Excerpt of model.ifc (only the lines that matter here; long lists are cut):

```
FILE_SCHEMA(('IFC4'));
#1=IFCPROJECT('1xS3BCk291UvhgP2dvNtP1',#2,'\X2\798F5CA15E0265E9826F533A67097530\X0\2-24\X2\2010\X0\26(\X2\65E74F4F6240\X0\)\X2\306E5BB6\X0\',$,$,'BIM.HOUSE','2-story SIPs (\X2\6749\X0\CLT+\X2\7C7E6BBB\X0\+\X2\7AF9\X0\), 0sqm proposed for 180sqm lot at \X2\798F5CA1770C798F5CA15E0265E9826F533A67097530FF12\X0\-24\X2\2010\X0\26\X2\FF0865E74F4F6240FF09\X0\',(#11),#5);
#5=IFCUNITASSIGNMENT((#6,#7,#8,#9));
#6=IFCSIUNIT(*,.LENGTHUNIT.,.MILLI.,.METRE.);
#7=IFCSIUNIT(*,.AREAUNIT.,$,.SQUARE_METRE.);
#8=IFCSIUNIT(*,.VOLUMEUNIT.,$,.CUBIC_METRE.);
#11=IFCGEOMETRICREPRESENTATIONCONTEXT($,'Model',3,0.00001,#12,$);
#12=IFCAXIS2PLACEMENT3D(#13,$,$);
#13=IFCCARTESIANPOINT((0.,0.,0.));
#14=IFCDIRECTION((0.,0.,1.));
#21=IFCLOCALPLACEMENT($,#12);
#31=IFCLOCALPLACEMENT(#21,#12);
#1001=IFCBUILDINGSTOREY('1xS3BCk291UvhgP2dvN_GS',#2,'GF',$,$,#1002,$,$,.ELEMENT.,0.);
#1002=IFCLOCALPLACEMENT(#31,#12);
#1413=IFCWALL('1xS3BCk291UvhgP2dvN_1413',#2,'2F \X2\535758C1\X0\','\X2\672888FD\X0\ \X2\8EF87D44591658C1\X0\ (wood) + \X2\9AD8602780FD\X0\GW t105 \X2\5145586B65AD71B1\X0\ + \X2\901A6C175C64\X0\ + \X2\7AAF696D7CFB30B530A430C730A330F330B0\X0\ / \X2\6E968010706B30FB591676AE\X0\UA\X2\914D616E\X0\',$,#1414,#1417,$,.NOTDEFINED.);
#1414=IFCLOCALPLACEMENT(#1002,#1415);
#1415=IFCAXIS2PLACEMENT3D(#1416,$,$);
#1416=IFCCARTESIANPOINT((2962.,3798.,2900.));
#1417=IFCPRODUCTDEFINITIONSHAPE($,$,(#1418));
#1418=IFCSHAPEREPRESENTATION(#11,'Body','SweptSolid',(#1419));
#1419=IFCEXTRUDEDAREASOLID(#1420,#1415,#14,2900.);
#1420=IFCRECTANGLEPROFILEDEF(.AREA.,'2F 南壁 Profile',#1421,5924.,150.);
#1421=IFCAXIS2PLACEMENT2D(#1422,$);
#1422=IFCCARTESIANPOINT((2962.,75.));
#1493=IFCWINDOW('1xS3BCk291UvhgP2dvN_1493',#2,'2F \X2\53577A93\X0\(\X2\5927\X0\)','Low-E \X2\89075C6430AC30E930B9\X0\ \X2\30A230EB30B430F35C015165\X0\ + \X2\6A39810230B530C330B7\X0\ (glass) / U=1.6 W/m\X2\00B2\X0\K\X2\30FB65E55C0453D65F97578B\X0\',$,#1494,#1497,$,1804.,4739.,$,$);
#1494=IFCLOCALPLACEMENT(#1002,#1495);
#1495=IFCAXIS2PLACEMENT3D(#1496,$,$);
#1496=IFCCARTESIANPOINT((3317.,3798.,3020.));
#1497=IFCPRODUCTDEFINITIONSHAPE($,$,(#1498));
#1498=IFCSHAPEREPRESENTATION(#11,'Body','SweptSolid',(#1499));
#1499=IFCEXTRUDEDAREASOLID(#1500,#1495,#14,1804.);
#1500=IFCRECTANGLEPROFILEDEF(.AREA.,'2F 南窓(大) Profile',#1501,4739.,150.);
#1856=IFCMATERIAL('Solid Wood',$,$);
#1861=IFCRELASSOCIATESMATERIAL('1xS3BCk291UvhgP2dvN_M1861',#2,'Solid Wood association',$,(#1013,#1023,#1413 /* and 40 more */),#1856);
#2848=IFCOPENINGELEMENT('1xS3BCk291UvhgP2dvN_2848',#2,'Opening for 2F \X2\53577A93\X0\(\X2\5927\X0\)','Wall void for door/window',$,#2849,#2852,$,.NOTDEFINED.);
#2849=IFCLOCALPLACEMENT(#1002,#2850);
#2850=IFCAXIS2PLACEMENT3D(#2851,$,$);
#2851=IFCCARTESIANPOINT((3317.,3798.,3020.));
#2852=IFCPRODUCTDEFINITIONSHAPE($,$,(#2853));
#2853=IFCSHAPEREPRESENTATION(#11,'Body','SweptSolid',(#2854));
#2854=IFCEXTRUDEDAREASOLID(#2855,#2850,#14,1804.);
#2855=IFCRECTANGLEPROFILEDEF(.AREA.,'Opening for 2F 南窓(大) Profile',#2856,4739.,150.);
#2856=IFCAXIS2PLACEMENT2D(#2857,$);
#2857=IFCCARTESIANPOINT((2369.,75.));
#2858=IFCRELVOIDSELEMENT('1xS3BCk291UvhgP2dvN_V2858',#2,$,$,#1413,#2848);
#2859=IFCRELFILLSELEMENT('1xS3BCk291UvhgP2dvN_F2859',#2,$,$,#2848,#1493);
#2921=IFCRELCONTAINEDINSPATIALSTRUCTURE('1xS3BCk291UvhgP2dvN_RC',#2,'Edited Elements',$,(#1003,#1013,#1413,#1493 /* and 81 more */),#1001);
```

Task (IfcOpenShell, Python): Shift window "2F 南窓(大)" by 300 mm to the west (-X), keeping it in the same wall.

```python
import ifcopenshell
import ifcopenshell.api.geometry
import ifcopenshell.util.placement

model = ifcopenshell.open("model.ifc")

window = model.by_guid("1xS3BCk291UvhgP2dvN_1493")
opening = window.FillsVoids[0].RelatingOpeningElement
wall = opening.VoidsElements[0].RelatingBuildingElement

wall_matrix = ifcopenshell.util.placement.get_local_placement(wall.ObjectPlacement)
shift = wall_matrix[:3, 0] * -300.0
before = ifcopenshell.util.placement.get_local_placement(window.ObjectPlacement)[:3, 3].copy()

# The window is not placed relative to its opening, so move both.
for product in (opening, window):
    matrix = ifcopenshell.util.placement.get_local_placement(product.ObjectPlacement)
    matrix[:3, 3] += shift
    ifcopenshell.api.geometry.edit_object_placement(model, product=product, matrix=matrix, is_si=False)

after = ifcopenshell.util.placement.get_local_placement(window.ObjectPlacement)[:3, 3]
print("window moved by", (after - before).round(3) + 0.0)

model.write("model-out.ifc")
```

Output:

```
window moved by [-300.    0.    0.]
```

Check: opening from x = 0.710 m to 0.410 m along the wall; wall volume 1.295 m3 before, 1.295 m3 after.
